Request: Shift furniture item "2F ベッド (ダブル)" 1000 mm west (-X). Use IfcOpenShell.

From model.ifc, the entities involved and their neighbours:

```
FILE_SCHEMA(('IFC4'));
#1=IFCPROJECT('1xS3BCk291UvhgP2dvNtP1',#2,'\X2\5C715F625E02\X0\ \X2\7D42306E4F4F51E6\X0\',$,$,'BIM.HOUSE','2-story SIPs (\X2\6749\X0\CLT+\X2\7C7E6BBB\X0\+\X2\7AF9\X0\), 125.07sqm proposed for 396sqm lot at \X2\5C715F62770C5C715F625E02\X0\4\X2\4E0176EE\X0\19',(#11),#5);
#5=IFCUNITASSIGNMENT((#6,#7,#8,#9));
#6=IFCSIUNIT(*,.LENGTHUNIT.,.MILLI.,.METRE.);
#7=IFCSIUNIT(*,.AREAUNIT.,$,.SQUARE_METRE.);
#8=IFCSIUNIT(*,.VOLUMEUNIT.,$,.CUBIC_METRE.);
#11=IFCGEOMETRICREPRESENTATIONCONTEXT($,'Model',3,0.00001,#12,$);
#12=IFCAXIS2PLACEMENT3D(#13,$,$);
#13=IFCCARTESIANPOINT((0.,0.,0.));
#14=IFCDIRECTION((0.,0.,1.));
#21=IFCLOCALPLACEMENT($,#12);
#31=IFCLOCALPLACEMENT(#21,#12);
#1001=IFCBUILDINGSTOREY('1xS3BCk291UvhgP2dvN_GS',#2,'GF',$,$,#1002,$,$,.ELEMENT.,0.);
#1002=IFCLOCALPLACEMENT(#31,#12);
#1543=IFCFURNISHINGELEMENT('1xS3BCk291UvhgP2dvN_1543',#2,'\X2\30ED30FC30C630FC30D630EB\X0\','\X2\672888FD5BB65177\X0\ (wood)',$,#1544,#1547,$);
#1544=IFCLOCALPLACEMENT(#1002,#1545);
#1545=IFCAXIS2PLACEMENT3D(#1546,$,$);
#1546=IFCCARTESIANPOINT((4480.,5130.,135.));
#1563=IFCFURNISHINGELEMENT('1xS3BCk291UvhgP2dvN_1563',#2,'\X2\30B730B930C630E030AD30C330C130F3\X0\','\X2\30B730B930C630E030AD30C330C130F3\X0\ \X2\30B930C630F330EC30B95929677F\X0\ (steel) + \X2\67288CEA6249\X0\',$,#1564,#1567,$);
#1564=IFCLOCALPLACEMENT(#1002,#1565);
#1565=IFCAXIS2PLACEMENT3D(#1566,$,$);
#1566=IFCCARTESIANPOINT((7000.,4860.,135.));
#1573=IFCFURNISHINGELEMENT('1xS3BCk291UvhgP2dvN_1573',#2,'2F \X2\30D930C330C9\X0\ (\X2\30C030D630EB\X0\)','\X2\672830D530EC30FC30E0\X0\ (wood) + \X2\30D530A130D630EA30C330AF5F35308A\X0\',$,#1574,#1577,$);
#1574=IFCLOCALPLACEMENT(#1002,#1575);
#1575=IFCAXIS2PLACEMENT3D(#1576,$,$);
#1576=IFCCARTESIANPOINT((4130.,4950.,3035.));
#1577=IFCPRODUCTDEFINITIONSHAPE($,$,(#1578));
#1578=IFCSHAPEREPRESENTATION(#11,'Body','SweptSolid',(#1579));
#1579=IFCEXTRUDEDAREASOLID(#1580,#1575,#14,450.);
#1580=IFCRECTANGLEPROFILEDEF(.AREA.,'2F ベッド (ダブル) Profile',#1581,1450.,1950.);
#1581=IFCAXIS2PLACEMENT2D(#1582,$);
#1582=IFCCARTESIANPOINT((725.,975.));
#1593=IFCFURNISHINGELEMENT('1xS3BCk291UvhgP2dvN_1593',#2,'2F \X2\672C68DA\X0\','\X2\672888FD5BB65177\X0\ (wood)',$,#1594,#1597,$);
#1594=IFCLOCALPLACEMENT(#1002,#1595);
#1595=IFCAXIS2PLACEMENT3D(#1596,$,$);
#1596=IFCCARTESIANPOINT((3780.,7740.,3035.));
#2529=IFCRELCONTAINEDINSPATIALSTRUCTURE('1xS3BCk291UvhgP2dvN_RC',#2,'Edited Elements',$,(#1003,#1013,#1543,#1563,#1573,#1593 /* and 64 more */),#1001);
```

```python
import ifcopenshell
import ifcopenshell.api.geometry
import ifcopenshell.util.placement

model = ifcopenshell.open("model.ifc")

item = model.by_id(1573)
matrix = ifcopenshell.util.placement.get_local_placement(item.ObjectPlacement)
matrix[0, 3] -= 1000.0
ifcopenshell.api.geometry.edit_object_placement(model, product=item, matrix=matrix, is_si=False)

print(ifcopenshell.util.placement.get_local_placement(item.ObjectPlacement).round(3) + 0.0)

model.write("model-out.ifc")
```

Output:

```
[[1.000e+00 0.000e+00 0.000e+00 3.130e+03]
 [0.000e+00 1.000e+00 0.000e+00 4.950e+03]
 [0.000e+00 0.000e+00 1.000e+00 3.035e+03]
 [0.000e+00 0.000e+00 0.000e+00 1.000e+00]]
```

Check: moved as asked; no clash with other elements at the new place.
